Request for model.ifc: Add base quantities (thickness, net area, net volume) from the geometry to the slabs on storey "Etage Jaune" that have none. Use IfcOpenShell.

First a look at what the model holds.

```python
import ifcopenshell
import ifcopenshell.util.element
import ifcopenshell.util.unit

model = ifcopenshell.open("model.ifc")
print(model.schema)
for unit_type in ("LENGTHUNIT", "AREAUNIT", "VOLUMEUNIT"):
    print(unit_type, ifcopenshell.util.unit.calculate_unit_scale(model, unit_type))
storey = next(s for s in model.by_type("IfcBuildingStorey") if s.Name == "Etage Jaune")
slabs = [e for e in ifcopenshell.util.element.get_decomposition(storey) if e.is_a("IfcSlab")]
for e in sorted(slabs, key=lambda e: e.id()):
    print(e.id(), e.is_a(), e.Name, list(ifcopenshell.util.element.get_psets(e, qtos_only=True)), sep=" | ")
```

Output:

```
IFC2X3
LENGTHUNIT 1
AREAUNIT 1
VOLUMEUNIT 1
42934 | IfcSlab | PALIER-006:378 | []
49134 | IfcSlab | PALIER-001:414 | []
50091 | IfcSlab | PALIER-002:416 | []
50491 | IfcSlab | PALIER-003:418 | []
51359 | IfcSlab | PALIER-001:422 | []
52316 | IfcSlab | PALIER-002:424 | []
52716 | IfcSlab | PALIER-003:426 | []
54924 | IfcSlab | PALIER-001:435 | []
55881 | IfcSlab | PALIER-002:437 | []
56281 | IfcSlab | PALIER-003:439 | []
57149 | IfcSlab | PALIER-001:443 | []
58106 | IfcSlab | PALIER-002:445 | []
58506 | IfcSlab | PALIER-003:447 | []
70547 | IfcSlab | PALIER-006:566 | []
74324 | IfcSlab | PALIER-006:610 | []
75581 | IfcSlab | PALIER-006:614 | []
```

```python
import ifcopenshell
import ifcopenshell.api.pset
import ifcopenshell.geom
import ifcopenshell.util.element
import ifcopenshell.util.shape
import ifcopenshell.util.unit

model = ifcopenshell.open("model.ifc")
unit_scale = ifcopenshell.util.unit.calculate_unit_scale(model)
area_scale = ifcopenshell.util.unit.calculate_unit_scale(model, "AREAUNIT")
volume_scale = ifcopenshell.util.unit.calculate_unit_scale(model, "VOLUMEUNIT")
settings = ifcopenshell.geom.settings()

storey = next(s for s in model.by_type("IfcBuildingStorey") if s.Name == "Etage Jaune")
slabs = [e for e in ifcopenshell.util.element.get_decomposition(storey) if e.is_a("IfcSlab")]

for e in sorted(slabs, key=lambda e: e.id()):
    if ifcopenshell.util.element.get_psets(e, qtos_only=True, should_inherit=False):
        continue
    # Geometry comes back in metres, in the element's own axes.
    shape = ifcopenshell.geom.create_shape(settings, e)
    values = {
        "Width": ifcopenshell.util.shape.get_z(shape.geometry) / unit_scale,
        "NetArea": ifcopenshell.util.shape.get_footprint_area(shape.geometry) / area_scale,
        "NetVolume": ifcopenshell.util.shape.get_volume(shape.geometry) / volume_scale,
    }
    qto = ifcopenshell.api.pset.add_qto(model, product=e, name="BaseQuantities")
    ifcopenshell.api.pset.edit_qto(model, qto=qto, properties=values)
    print(e.id(), {k: round(v, 3) for k, v in values.items()})

model.write("model_v2.ifc")
```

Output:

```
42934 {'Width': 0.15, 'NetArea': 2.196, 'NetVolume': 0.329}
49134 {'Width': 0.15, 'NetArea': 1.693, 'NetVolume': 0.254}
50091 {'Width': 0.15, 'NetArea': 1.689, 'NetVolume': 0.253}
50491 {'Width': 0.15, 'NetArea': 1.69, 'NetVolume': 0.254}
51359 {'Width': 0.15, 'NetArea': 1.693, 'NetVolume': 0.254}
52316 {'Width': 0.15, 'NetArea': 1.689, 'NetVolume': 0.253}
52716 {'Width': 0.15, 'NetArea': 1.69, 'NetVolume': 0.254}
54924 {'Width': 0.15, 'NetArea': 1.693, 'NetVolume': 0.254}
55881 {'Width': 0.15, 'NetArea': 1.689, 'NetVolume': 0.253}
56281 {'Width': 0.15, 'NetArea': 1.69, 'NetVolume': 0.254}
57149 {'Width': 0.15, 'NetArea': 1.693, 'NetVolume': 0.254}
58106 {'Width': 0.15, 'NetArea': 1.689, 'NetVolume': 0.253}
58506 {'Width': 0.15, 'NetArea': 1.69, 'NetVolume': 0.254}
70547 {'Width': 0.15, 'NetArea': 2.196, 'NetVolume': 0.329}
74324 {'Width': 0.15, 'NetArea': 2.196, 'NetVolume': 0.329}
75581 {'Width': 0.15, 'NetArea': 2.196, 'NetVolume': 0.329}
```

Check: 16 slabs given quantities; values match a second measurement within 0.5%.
